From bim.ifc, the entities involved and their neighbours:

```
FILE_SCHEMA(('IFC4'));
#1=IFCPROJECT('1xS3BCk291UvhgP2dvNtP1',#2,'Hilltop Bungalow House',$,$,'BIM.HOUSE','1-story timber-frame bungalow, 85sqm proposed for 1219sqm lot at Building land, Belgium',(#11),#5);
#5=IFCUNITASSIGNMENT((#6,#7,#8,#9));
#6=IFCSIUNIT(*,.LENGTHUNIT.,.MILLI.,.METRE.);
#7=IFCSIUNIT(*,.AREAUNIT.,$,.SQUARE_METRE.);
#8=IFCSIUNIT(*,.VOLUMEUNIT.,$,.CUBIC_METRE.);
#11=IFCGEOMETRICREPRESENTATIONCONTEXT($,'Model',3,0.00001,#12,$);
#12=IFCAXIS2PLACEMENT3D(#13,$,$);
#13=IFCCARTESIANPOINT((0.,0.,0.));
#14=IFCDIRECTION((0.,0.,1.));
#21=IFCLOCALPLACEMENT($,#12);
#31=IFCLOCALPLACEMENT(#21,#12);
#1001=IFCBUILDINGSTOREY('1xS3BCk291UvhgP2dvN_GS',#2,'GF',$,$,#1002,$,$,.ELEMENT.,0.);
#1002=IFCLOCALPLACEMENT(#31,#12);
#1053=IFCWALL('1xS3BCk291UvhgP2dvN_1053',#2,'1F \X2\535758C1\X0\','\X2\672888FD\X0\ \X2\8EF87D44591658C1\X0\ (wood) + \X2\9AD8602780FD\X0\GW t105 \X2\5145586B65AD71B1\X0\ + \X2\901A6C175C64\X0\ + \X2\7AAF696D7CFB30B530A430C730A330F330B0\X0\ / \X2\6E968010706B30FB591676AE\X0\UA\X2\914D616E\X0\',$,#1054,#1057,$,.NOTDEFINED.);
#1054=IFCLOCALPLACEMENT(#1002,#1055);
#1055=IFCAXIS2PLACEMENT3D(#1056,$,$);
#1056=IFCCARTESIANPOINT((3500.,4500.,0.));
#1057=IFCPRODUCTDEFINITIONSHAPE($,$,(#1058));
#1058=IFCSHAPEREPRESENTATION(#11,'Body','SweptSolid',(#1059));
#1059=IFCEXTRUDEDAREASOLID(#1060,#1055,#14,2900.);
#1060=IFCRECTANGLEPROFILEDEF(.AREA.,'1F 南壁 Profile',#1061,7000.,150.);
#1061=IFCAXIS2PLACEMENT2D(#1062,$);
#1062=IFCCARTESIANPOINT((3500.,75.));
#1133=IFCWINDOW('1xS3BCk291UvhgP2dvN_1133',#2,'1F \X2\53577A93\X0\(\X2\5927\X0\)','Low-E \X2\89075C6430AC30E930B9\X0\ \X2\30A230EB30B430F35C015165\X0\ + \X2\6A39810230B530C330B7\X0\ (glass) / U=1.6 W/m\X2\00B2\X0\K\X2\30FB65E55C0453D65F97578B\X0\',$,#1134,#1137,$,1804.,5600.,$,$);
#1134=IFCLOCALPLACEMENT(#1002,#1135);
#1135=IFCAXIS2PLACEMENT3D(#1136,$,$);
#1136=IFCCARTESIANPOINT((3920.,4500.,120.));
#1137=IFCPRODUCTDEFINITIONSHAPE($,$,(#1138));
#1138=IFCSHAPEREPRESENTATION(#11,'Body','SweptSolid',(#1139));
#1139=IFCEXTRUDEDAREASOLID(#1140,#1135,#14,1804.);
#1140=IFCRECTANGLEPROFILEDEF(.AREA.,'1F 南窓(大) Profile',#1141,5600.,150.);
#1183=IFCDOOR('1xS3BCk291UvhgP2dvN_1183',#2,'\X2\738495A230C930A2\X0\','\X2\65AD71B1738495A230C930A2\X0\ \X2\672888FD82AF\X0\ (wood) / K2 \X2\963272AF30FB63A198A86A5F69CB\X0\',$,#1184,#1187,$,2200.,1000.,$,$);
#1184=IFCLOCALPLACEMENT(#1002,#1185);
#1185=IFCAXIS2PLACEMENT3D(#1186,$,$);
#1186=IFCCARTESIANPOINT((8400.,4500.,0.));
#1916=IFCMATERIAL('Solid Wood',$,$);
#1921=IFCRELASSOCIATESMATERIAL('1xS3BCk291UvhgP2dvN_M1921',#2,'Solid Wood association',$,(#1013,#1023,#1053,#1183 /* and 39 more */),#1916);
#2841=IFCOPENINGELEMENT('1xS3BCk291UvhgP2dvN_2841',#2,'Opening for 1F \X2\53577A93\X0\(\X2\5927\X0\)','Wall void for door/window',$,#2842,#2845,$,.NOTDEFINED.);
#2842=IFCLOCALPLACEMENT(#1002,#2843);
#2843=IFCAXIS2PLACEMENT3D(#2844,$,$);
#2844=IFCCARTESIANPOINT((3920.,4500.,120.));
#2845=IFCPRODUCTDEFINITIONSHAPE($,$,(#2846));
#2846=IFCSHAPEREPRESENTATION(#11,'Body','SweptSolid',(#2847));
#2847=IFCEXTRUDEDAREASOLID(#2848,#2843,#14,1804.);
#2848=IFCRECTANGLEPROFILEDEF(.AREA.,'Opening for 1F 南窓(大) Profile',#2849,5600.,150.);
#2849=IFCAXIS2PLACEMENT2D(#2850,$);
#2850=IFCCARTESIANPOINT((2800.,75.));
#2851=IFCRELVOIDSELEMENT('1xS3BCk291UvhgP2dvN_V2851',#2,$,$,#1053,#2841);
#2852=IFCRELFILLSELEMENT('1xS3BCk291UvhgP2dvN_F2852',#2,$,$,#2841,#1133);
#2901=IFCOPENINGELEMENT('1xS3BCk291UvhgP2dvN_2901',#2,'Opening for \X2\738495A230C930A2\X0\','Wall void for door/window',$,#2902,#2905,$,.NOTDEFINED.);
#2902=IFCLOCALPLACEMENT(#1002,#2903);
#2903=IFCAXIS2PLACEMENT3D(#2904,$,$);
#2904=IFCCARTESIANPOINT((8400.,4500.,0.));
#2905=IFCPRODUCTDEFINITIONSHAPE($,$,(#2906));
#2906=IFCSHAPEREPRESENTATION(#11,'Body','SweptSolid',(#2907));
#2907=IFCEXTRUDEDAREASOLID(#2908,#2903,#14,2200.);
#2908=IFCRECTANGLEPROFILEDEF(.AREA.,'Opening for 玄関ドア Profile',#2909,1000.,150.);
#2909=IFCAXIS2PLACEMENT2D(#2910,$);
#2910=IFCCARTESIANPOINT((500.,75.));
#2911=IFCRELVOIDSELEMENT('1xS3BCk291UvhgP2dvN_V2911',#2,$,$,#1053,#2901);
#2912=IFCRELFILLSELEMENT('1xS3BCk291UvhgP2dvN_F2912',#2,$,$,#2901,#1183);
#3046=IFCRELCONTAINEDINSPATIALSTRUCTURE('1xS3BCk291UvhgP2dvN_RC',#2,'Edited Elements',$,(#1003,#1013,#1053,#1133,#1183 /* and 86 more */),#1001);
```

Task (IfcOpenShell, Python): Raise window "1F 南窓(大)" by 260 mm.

```python
import numpy as np
import ifcopenshell
import ifcopenshell.api.geometry
import ifcopenshell.util.placement
import ifcopenshell.util.unit

model = ifcopenshell.open("bim.ifc")
unit_scale = ifcopenshell.util.unit.calculate_unit_scale(model)

window = model.by_guid("1xS3BCk291UvhgP2dvN_1133")
opening = window.FillsVoids[0].RelatingOpeningElement
dz = 0.26 / unit_scale

shift = np.array([0.0, 0.0, dz])
# The window is not placed relative to its opening, so move both.
for product in (opening, window):
    matrix = ifcopenshell.util.placement.get_local_placement(product.ObjectPlacement)
    matrix[:3, 3] += shift
    ifcopenshell.api.geometry.edit_object_placement(model, product=product, matrix=matrix, is_si=False)

print(f"moved by {dz * unit_scale:+.3f} m")

model.write("bim_rev.ifc")
```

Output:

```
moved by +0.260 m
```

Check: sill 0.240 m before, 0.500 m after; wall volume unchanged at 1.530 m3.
